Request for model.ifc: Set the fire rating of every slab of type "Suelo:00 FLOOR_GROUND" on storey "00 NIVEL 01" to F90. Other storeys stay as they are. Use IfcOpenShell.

First a look at what the model holds.

```python
import ifcopenshell
import ifcopenshell.util.element

model = ifcopenshell.open("model.ifc")
print(model.schema)
storey = next(s for s in model.by_type("IfcBuildingStorey") if s.Name == "00 NIVEL 01")
slabs = [e for e in ifcopenshell.util.element.get_decomposition(storey) if e.is_a("IfcSlab")]
seen = {}
for e in slabs:
    element_type = ifcopenshell.util.element.get_type(e)
    key = (element_type.Name if element_type != e and element_type else None, ifcopenshell.util.element.get_pset(e, "Pset_SlabCommon", "FireRating"))
    seen[key] = seen.get(key, 0) + 1
for (name, value), count in sorted(seen.items(), key=str):
    print(count, "x", name, "|", value)
```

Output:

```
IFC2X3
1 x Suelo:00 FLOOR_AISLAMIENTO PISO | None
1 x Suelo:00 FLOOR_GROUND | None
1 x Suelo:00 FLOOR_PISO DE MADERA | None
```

```python
import ifcopenshell
import ifcopenshell.api.pset
import ifcopenshell.util.element

model = ifcopenshell.open("model.ifc")

storey = next(s for s in model.by_type("IfcBuildingStorey") if s.Name == "00 NIVEL 01")
slabs = [e for e in ifcopenshell.util.element.get_decomposition(storey) if e.is_a("IfcSlab")]

count = 0
for e in slabs:
    element_type = ifcopenshell.util.element.get_type(e)
    if element_type in (None, e) or element_type.Name != "Suelo:00 FLOOR_GROUND":
        continue
    # add_pset returns the element's existing set when there is one.
    pset = ifcopenshell.api.pset.add_pset(model, product=e, name="Pset_SlabCommon")
    ifcopenshell.api.pset.edit_pset(model, pset=pset, properties={"FireRating": "F90"})
    count += 1

print(count, "slabs updated")

model.write("model-out.ifc")
```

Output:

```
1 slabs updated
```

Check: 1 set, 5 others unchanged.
